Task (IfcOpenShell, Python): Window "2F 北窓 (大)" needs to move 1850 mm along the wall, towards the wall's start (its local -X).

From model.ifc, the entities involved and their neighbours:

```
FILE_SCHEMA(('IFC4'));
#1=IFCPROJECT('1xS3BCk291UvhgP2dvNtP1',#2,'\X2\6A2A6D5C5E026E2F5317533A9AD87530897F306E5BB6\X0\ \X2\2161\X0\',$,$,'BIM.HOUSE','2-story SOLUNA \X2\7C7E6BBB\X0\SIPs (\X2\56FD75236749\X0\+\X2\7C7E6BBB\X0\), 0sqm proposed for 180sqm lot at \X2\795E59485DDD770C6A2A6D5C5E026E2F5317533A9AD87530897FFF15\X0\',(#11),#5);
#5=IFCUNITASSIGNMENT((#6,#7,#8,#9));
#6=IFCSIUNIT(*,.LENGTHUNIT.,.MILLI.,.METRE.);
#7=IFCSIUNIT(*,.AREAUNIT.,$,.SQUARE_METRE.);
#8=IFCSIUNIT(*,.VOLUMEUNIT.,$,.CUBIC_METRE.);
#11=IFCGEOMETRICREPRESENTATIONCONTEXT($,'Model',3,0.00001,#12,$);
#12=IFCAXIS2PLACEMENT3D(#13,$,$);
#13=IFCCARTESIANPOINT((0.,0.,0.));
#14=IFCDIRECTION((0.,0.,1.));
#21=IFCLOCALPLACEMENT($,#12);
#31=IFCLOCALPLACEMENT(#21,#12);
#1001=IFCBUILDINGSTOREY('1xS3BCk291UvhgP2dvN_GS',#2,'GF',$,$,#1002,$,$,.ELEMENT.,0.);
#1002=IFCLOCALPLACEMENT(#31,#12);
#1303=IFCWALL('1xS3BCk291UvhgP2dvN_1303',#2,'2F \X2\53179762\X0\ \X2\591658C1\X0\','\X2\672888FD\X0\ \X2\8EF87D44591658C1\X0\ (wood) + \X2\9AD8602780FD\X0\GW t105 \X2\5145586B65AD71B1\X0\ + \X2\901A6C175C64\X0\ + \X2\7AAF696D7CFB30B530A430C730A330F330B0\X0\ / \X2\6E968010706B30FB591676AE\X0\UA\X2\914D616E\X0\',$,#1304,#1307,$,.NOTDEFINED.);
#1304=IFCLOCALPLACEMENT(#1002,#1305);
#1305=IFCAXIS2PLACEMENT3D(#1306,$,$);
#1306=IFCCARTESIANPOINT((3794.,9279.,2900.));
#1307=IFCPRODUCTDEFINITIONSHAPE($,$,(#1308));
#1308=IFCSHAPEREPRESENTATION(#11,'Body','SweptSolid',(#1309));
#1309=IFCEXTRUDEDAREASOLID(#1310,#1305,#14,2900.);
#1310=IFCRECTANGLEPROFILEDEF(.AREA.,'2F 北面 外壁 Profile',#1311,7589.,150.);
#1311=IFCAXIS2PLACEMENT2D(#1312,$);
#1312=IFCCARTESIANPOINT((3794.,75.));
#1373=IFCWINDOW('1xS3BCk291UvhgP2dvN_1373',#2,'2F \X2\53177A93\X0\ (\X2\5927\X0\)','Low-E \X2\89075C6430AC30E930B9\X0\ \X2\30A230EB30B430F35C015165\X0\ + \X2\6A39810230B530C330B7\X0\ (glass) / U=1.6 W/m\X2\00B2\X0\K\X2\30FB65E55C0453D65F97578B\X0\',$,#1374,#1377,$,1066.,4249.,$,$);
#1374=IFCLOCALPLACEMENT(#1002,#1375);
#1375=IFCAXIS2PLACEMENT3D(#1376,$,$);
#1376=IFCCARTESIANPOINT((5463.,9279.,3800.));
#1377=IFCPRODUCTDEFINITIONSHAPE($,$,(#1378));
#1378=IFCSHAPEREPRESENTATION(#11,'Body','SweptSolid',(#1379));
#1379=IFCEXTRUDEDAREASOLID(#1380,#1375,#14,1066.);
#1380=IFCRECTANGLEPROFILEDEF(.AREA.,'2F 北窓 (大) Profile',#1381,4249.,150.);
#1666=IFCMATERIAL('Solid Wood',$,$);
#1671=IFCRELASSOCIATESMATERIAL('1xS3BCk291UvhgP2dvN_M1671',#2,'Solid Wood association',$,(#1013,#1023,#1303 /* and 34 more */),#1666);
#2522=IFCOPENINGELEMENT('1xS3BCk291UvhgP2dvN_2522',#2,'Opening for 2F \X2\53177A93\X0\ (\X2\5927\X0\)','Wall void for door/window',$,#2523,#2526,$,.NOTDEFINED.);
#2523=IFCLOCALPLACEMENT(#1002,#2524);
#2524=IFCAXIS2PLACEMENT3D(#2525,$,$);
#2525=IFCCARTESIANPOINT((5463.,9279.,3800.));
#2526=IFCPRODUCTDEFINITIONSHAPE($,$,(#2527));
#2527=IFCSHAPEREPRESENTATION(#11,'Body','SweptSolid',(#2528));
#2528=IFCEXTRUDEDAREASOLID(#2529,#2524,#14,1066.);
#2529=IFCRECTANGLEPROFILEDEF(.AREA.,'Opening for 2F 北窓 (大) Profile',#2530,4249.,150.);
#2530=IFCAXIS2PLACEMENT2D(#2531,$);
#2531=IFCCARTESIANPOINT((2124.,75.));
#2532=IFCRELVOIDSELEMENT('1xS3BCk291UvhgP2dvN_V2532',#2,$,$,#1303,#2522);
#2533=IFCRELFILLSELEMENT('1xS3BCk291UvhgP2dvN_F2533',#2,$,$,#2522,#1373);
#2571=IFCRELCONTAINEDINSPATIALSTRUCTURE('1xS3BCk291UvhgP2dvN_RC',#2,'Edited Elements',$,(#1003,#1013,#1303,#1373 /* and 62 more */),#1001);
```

```python
import ifcopenshell
import ifcopenshell.api.geometry
import ifcopenshell.util.placement

model = ifcopenshell.open("model.ifc")

window = model.by_id(1373)
opening = window.FillsVoids[0].RelatingOpeningElement
wall = opening.VoidsElements[0].RelatingBuildingElement

wall_matrix = ifcopenshell.util.placement.get_local_placement(wall.ObjectPlacement)
shift = wall_matrix[:3, 0] * -1850.0
before = ifcopenshell.util.placement.get_local_placement(window.ObjectPlacement)[:3, 3].copy()

# The window is not placed relative to its opening, so move both.
for product in (opening, window):
    matrix = ifcopenshell.util.placement.get_local_placement(product.ObjectPlacement)
    matrix[:3, 3] += shift
    ifcopenshell.api.geometry.edit_object_placement(model, product=product, matrix=matrix, is_si=False)

after = ifcopenshell.util.placement.get_local_placement(window.ObjectPlacement)[:3, 3]
print("window moved by", (after - before).round(3) + 0.0)

model.write("model_rev.ifc")
```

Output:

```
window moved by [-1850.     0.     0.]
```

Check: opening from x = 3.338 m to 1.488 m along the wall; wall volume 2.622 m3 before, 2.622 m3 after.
